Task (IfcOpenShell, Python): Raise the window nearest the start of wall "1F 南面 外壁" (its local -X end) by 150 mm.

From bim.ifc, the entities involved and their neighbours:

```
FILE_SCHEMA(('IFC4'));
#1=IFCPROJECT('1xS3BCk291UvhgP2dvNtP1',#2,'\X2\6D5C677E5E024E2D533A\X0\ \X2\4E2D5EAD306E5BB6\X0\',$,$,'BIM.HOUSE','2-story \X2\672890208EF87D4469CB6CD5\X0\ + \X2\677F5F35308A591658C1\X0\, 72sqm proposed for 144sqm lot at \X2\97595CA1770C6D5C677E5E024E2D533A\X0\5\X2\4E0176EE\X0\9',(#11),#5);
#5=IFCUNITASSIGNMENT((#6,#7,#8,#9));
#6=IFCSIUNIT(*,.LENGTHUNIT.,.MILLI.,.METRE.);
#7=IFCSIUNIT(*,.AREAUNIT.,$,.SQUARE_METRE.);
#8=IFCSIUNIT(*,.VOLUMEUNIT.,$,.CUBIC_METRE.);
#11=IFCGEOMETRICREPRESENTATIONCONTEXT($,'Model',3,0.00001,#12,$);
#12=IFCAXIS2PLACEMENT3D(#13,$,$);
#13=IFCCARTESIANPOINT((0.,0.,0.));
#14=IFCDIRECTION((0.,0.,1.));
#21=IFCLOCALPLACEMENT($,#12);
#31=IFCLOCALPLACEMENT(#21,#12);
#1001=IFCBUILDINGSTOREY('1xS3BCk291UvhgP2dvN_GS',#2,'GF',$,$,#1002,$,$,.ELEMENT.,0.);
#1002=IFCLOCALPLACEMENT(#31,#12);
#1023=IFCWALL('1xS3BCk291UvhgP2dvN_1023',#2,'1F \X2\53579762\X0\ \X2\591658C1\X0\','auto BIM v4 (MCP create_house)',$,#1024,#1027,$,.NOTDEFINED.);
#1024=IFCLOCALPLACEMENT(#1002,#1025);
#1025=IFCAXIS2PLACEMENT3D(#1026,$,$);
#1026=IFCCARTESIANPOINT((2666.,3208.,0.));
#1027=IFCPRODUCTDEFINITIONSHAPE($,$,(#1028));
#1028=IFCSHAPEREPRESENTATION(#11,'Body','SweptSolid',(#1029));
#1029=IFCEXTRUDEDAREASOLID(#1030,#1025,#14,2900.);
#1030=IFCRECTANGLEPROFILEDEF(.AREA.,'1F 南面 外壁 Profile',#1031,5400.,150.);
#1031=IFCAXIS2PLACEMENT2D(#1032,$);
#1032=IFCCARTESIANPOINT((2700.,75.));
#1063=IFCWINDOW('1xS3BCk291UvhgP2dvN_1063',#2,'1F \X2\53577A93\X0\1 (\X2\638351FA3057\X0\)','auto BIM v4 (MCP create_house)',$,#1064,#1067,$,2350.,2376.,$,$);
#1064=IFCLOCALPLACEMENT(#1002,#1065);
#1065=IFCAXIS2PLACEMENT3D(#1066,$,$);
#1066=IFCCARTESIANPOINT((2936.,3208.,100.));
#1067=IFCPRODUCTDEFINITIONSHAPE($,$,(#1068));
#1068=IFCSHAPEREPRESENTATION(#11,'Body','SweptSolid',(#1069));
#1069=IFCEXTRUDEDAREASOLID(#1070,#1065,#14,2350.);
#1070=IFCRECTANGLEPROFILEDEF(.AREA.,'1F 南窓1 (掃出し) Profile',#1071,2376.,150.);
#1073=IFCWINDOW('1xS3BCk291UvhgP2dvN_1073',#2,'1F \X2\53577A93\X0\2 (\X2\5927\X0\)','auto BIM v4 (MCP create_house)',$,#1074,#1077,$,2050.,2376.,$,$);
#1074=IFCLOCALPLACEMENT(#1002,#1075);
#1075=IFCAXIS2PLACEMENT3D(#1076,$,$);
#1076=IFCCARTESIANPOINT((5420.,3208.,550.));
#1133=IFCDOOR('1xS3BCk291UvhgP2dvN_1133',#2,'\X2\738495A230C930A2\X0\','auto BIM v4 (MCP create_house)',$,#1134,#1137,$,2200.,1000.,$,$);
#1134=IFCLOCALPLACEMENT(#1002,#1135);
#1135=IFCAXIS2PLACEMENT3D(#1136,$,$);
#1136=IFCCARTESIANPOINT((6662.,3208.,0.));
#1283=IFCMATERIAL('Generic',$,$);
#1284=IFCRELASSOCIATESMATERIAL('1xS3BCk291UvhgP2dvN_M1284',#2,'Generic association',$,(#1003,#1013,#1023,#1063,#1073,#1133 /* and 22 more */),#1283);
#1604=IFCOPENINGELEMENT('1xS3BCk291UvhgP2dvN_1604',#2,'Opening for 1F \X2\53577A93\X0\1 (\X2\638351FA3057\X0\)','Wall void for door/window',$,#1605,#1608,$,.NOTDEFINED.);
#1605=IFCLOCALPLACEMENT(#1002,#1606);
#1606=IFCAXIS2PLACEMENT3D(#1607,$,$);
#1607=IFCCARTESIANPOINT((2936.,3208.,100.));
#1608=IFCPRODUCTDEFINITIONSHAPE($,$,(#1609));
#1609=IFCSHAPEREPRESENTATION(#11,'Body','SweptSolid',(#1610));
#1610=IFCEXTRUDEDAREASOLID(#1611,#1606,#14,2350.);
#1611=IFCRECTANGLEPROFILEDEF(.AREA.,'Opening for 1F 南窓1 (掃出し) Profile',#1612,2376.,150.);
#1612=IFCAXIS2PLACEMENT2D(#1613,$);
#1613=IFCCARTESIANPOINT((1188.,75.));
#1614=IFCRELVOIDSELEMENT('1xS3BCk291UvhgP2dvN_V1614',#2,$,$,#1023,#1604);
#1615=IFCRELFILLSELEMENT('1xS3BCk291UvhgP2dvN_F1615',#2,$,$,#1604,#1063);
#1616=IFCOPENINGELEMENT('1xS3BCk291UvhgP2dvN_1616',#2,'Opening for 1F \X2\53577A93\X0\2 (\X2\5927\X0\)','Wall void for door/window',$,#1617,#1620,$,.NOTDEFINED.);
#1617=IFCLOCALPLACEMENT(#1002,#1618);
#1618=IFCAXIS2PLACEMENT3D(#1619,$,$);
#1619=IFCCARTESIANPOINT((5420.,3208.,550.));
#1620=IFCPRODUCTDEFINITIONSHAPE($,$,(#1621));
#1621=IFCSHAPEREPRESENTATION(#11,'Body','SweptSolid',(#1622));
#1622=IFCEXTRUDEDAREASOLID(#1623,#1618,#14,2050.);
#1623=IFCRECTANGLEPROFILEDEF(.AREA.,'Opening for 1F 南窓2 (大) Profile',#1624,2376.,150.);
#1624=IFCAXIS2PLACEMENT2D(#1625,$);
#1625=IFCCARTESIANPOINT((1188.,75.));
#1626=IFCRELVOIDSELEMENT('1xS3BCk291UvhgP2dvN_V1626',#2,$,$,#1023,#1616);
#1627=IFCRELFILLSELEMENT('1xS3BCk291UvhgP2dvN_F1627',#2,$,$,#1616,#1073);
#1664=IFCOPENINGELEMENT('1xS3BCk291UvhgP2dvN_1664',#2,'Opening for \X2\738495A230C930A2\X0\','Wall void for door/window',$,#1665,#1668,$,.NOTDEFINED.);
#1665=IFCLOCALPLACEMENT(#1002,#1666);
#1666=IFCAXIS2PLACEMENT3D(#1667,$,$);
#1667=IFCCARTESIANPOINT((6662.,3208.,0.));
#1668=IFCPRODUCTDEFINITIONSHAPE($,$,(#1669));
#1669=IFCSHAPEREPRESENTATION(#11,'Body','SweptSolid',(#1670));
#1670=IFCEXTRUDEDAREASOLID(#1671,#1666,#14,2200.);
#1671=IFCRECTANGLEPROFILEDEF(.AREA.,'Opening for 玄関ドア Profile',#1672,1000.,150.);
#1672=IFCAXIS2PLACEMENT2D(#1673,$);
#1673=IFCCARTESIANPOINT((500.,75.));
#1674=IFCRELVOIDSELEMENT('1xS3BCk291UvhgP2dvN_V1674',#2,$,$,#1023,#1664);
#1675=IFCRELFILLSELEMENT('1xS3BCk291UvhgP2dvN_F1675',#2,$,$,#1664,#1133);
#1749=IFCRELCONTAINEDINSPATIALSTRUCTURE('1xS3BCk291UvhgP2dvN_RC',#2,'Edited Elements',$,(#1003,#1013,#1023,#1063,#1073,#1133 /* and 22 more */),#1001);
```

```python
import numpy as np
import ifcopenshell
import ifcopenshell.api.geometry
import ifcopenshell.util.placement
import ifcopenshell.util.unit

model = ifcopenshell.open("bim.ifc")
unit_scale = ifcopenshell.util.unit.calculate_unit_scale(model)

window = model.by_guid("1xS3BCk291UvhgP2dvN_1063")
opening = window.FillsVoids[0].RelatingOpeningElement
dz = 0.15 / unit_scale

shift = np.array([0.0, 0.0, dz])
# The window is not placed relative to its opening, so move both.
for product in (opening, window):
    matrix = ifcopenshell.util.placement.get_local_placement(product.ObjectPlacement)
    matrix[:3, 3] += shift
    ifcopenshell.api.geometry.edit_object_placement(model, product=product, matrix=matrix, is_si=False)

print(f"moved by {dz * unit_scale:+.3f} m")

model.write("bim_updated.ifc")
```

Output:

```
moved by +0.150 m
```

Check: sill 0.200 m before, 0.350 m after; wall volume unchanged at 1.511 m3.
